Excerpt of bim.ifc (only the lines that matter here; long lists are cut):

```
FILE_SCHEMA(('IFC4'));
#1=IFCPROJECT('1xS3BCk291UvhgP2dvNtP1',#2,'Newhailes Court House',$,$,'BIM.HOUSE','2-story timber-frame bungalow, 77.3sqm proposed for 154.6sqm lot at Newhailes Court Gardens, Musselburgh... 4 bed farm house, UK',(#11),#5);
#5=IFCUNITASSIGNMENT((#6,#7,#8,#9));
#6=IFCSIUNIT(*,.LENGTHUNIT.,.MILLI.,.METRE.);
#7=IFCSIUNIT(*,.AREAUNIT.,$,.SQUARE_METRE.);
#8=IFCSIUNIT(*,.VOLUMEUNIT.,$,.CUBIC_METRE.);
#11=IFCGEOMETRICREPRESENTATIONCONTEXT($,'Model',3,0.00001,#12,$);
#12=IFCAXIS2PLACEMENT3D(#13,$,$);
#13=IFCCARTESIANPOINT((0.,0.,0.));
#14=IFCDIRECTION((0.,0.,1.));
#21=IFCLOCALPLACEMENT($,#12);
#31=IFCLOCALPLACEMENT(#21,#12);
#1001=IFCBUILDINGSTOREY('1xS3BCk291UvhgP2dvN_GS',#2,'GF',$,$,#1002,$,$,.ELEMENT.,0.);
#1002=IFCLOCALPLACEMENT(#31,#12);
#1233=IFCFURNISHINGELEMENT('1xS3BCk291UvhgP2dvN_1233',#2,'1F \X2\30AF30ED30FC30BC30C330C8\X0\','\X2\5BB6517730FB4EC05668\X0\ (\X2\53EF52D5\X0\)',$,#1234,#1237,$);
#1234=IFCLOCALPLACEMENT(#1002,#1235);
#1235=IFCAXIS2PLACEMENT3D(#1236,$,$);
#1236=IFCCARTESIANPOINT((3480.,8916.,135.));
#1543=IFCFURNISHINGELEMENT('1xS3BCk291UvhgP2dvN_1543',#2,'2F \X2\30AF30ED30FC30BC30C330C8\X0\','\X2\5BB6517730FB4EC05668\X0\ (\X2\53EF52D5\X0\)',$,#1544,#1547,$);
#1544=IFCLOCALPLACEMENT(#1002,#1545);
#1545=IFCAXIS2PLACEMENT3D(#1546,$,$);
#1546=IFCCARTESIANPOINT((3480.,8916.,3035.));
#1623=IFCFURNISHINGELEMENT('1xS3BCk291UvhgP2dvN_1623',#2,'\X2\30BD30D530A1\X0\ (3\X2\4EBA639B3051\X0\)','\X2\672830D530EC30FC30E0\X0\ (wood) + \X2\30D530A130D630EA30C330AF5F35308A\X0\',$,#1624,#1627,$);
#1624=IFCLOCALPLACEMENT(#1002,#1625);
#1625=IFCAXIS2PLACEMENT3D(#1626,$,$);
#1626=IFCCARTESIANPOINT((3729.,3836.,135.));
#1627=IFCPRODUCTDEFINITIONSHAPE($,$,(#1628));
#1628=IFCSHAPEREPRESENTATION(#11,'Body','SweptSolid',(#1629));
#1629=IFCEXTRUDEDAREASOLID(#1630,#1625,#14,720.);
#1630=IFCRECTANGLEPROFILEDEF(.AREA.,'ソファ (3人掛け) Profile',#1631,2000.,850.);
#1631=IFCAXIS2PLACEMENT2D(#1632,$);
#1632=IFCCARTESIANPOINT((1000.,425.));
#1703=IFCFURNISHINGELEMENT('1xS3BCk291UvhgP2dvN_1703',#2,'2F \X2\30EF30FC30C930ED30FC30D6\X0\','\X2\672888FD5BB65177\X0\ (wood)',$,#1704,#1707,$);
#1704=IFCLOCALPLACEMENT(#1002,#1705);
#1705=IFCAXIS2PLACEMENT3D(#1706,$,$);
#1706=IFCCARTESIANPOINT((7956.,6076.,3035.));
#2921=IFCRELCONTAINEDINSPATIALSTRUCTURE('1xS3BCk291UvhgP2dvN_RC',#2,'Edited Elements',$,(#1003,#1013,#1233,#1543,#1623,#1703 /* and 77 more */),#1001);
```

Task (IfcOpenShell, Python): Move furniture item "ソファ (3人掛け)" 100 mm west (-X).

```python
import ifcopenshell
import ifcopenshell.api.geometry
import ifcopenshell.util.placement
import ifcopenshell.util.unit

model = ifcopenshell.open("bim.ifc")
unit_scale = ifcopenshell.util.unit.calculate_unit_scale(model)

item = model.by_guid("1xS3BCk291UvhgP2dvN_1623")
matrix = ifcopenshell.util.placement.get_local_placement(item.ObjectPlacement)
matrix[0, 3] -= 0.1 / unit_scale
ifcopenshell.api.geometry.edit_object_placement(model, product=item, matrix=matrix, is_si=False)

print(ifcopenshell.util.placement.get_local_placement(item.ObjectPlacement).round(3) + 0.0)

model.write("bim_edited.ifc")
```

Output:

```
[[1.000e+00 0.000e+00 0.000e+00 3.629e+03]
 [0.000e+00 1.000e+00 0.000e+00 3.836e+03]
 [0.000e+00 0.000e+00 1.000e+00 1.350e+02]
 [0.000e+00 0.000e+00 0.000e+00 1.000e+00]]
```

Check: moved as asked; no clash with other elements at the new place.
